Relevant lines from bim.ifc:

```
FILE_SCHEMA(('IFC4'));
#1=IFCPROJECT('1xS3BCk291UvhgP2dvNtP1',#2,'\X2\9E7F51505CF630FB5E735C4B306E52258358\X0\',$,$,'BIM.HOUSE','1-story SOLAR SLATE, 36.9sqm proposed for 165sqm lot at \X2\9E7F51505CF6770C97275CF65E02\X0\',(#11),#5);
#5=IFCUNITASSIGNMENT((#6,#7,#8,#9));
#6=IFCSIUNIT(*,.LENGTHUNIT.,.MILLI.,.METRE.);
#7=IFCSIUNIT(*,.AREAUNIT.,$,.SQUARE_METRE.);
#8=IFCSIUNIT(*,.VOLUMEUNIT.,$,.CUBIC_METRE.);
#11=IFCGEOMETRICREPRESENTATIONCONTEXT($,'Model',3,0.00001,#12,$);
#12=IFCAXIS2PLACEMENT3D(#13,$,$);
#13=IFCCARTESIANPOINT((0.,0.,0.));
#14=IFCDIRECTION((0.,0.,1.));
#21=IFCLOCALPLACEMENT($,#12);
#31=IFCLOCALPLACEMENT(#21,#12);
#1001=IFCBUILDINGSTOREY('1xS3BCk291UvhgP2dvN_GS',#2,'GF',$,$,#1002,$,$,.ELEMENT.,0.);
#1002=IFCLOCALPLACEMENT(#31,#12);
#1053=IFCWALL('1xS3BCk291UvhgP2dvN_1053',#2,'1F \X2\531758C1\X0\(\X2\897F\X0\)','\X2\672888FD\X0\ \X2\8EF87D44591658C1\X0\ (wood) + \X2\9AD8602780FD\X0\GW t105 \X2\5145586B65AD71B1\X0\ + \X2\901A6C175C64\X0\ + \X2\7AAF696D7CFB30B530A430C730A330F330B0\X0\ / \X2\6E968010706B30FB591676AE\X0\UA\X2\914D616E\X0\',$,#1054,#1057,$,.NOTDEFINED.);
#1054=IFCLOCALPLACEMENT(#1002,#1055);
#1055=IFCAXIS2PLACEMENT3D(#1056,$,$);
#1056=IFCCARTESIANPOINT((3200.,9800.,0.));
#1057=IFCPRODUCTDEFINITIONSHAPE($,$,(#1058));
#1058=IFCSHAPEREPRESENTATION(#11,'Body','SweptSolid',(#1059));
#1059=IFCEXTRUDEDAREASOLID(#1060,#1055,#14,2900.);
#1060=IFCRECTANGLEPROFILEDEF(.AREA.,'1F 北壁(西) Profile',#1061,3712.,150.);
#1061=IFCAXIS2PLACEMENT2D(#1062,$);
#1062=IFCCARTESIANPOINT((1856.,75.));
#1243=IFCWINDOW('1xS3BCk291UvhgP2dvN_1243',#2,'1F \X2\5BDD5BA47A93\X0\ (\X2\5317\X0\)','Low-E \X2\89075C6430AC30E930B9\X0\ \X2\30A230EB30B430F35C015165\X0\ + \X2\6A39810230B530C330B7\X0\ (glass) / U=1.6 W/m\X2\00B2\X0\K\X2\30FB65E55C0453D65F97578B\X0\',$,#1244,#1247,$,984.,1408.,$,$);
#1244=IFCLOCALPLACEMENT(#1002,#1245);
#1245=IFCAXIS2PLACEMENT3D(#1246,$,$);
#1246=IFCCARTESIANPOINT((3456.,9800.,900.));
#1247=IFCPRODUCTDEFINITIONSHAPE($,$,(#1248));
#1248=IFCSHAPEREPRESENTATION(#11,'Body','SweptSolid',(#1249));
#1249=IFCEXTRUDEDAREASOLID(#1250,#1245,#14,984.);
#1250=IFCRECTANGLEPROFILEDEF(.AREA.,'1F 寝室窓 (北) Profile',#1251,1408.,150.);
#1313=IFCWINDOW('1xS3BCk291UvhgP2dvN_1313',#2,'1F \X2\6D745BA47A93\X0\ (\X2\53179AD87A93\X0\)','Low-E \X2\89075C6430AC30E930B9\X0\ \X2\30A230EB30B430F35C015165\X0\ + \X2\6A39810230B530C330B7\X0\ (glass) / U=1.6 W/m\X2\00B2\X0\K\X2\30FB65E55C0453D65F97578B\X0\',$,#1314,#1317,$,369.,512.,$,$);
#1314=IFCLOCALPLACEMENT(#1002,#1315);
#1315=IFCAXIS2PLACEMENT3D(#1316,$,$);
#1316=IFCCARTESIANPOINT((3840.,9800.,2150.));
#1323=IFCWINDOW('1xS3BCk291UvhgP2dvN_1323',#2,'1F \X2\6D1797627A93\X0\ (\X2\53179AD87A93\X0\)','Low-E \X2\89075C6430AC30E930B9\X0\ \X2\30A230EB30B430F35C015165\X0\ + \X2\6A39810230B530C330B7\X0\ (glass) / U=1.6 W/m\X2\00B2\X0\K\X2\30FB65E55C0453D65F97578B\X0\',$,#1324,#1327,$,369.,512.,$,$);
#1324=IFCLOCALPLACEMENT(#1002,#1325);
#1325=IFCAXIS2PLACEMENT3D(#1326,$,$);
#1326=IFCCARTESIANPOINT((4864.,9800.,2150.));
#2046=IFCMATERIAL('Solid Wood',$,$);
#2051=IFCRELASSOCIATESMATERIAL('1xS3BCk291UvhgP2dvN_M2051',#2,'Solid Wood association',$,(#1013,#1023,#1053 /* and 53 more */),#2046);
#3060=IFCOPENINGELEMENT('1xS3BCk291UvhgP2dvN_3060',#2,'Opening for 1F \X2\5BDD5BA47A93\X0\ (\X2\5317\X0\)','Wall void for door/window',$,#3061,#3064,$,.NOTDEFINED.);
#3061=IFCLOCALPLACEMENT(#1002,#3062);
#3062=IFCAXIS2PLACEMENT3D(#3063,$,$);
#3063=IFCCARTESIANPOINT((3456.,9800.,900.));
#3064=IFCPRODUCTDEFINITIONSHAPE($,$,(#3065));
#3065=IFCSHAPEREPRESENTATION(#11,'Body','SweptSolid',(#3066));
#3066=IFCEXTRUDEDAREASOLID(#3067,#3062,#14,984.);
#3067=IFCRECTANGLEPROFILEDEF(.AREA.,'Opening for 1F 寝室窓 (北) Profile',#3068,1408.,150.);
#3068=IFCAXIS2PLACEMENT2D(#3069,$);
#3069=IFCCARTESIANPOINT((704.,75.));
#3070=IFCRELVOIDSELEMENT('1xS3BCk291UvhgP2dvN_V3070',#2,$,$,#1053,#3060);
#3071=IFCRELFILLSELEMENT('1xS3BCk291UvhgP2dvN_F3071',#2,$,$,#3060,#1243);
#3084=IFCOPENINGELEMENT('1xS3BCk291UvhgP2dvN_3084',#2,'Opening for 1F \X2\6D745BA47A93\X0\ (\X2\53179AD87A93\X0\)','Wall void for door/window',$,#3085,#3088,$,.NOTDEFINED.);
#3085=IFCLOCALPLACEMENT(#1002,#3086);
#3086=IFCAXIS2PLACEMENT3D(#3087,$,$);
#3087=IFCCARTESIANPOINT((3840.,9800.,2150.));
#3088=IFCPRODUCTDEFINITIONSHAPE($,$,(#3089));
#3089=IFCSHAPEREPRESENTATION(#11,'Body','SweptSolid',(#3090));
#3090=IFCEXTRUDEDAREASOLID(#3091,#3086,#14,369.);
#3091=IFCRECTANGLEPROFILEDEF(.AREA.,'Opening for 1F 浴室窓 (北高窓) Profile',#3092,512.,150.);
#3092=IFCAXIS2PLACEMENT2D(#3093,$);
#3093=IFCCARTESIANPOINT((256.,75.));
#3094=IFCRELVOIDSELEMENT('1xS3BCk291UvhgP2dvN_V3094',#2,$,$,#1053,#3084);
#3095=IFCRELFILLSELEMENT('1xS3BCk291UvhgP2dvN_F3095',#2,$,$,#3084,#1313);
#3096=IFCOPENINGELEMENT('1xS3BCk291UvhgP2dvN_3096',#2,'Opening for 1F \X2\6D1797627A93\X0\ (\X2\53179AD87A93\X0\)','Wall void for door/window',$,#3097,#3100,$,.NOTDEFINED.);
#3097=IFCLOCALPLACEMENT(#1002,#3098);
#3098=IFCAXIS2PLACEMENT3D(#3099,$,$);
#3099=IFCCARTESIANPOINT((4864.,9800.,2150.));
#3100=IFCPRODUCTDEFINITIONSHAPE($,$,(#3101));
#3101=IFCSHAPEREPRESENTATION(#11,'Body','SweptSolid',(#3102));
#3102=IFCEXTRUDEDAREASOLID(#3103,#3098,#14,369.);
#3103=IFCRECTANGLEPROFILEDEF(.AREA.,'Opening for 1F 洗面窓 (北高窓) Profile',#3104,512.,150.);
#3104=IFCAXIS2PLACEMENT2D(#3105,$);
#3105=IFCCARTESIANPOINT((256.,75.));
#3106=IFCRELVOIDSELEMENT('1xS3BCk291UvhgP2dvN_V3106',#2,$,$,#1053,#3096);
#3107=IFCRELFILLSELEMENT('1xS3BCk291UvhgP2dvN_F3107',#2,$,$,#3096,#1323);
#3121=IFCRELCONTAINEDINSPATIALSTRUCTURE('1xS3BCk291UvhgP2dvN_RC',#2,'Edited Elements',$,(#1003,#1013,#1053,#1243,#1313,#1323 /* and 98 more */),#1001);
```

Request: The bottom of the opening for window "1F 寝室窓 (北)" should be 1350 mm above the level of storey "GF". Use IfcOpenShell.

```python
import numpy as np
import ifcopenshell
import ifcopenshell.api.geometry
import ifcopenshell.geom
import ifcopenshell.util.element
import ifcopenshell.util.placement
import ifcopenshell.util.shape
import ifcopenshell.util.unit

model = ifcopenshell.open("bim.ifc")
unit_scale = ifcopenshell.util.unit.calculate_unit_scale(model)

window = model.by_guid("1xS3BCk291UvhgP2dvN_1243")
opening = window.FillsVoids[0].RelatingOpeningElement
storey = ifcopenshell.util.element.get_container(window, ifc_class="IfcBuildingStorey")
level = ifcopenshell.util.placement.get_local_placement(storey.ObjectPlacement)[2, 3]

# The opening's origin need not be at the sill, so measure its lowest point.
shape = ifcopenshell.geom.create_shape(ifcopenshell.geom.settings(), opening)
bottom = ifcopenshell.util.shape.get_shape_bottom_elevation(shape, shape.geometry) / unit_scale
dz = level + 1.35 / unit_scale - bottom

shift = np.array([0.0, 0.0, dz])
# The window is not placed relative to its opening, so move both.
for product in (opening, window):
    matrix = ifcopenshell.util.placement.get_local_placement(product.ObjectPlacement)
    matrix[:3, 3] += shift
    ifcopenshell.api.geometry.edit_object_placement(model, product=product, matrix=matrix, is_si=False)

print(f"moved by {dz * unit_scale:+.3f} m")

model.write("bim_edited.ifc")
```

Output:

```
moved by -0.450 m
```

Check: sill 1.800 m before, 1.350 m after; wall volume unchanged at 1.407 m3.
